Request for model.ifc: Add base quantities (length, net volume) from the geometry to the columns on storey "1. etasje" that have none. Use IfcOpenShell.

First a look at what the model holds.

```python
import ifcopenshell
import ifcopenshell.util.element
import ifcopenshell.util.unit

model = ifcopenshell.open("model.ifc")
print(model.schema)
for unit_type in ("LENGTHUNIT", "AREAUNIT", "VOLUMEUNIT"):
    print(unit_type, ifcopenshell.util.unit.calculate_unit_scale(model, unit_type))
storey = next(s for s in model.by_type("IfcBuildingStorey") if s.Name == "1. etasje")
columns = [e for e in ifcopenshell.util.element.get_decomposition(storey) if e.is_a("IfcColumn")]
for e in sorted(columns, key=lambda e: e.id()):
    print(e.id(), e.is_a(), e.Name, list(ifcopenshell.util.element.get_psets(e, qtos_only=True)), sep=" | ")
```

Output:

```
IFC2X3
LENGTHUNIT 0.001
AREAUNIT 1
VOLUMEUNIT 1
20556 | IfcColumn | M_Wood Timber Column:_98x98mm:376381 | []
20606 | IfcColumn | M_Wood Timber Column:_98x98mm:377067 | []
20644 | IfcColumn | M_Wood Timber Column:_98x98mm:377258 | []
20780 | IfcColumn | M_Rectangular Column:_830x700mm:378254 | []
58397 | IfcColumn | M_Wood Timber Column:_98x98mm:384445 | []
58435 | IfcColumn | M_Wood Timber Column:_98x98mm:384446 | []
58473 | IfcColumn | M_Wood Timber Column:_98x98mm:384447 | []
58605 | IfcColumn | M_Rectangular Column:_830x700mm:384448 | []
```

```python
import ifcopenshell
import ifcopenshell.api.pset
import ifcopenshell.geom
import ifcopenshell.util.element
import ifcopenshell.util.shape
import ifcopenshell.util.unit

model = ifcopenshell.open("model.ifc")
unit_scale = ifcopenshell.util.unit.calculate_unit_scale(model)
volume_scale = ifcopenshell.util.unit.calculate_unit_scale(model, "VOLUMEUNIT")
settings = ifcopenshell.geom.settings()

storey = next(s for s in model.by_type("IfcBuildingStorey") if s.Name == "1. etasje")
columns = [e for e in ifcopenshell.util.element.get_decomposition(storey) if e.is_a("IfcColumn")]

for e in sorted(columns, key=lambda e: e.id()):
    if ifcopenshell.util.element.get_psets(e, qtos_only=True, should_inherit=False):
        continue
    # Geometry comes back in metres, in the element's own axes.
    shape = ifcopenshell.geom.create_shape(settings, e)
    values = {
        "Length": ifcopenshell.util.shape.get_z(shape.geometry) / unit_scale,
        "NetVolume": ifcopenshell.util.shape.get_volume(shape.geometry) / volume_scale,
    }
    qto = ifcopenshell.api.pset.add_qto(model, product=e, name="BaseQuantities")
    ifcopenshell.api.pset.edit_qto(model, qto=qto, properties=values)
    print(e.id(), {k: round(v, 3) for k, v in values.items()})

model.write("model-out.ifc")
```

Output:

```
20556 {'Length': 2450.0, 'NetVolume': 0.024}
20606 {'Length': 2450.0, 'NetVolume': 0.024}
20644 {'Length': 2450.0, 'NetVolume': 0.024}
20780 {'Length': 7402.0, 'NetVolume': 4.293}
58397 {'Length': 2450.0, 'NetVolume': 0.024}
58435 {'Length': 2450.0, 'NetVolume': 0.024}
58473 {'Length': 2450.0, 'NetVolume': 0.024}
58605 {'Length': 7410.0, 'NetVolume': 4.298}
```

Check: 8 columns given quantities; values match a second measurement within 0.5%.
